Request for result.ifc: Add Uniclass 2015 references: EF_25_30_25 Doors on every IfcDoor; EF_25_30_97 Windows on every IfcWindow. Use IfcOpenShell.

First a look at what the model holds.

```python
import ifcopenshell

model = ifcopenshell.open("result.ifc")
print(model.schema)
print("classifications:", [c.Name for c in model.by_type("IfcClassification")])
for ifc_class in ("IfcDoor", "IfcRoof", "IfcStair", "IfcWall", "IfcWindow"):
    print(ifc_class, len(model.by_type(ifc_class)))
```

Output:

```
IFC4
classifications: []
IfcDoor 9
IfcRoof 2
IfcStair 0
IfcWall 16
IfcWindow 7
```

```python
import ifcopenshell
import ifcopenshell.api.classification

model = ifcopenshell.open("result.ifc")

system = ifcopenshell.api.classification.add_classification(model, classification="Uniclass 2015")

codes = {
    "IfcDoor": ("EF_25_30_25", "Doors"),
    "IfcWindow": ("EF_25_30_97", "Windows"),
}
for ifc_class, (code, name) in codes.items():
    products = model.by_type(ifc_class)
    ifcopenshell.api.classification.add_reference(
        model, products=products, classification=system, identification=code, name=name
    )
    print(code, len(products))

model.write("result_edited.ifc")
```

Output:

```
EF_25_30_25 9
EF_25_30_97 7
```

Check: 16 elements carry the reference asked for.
